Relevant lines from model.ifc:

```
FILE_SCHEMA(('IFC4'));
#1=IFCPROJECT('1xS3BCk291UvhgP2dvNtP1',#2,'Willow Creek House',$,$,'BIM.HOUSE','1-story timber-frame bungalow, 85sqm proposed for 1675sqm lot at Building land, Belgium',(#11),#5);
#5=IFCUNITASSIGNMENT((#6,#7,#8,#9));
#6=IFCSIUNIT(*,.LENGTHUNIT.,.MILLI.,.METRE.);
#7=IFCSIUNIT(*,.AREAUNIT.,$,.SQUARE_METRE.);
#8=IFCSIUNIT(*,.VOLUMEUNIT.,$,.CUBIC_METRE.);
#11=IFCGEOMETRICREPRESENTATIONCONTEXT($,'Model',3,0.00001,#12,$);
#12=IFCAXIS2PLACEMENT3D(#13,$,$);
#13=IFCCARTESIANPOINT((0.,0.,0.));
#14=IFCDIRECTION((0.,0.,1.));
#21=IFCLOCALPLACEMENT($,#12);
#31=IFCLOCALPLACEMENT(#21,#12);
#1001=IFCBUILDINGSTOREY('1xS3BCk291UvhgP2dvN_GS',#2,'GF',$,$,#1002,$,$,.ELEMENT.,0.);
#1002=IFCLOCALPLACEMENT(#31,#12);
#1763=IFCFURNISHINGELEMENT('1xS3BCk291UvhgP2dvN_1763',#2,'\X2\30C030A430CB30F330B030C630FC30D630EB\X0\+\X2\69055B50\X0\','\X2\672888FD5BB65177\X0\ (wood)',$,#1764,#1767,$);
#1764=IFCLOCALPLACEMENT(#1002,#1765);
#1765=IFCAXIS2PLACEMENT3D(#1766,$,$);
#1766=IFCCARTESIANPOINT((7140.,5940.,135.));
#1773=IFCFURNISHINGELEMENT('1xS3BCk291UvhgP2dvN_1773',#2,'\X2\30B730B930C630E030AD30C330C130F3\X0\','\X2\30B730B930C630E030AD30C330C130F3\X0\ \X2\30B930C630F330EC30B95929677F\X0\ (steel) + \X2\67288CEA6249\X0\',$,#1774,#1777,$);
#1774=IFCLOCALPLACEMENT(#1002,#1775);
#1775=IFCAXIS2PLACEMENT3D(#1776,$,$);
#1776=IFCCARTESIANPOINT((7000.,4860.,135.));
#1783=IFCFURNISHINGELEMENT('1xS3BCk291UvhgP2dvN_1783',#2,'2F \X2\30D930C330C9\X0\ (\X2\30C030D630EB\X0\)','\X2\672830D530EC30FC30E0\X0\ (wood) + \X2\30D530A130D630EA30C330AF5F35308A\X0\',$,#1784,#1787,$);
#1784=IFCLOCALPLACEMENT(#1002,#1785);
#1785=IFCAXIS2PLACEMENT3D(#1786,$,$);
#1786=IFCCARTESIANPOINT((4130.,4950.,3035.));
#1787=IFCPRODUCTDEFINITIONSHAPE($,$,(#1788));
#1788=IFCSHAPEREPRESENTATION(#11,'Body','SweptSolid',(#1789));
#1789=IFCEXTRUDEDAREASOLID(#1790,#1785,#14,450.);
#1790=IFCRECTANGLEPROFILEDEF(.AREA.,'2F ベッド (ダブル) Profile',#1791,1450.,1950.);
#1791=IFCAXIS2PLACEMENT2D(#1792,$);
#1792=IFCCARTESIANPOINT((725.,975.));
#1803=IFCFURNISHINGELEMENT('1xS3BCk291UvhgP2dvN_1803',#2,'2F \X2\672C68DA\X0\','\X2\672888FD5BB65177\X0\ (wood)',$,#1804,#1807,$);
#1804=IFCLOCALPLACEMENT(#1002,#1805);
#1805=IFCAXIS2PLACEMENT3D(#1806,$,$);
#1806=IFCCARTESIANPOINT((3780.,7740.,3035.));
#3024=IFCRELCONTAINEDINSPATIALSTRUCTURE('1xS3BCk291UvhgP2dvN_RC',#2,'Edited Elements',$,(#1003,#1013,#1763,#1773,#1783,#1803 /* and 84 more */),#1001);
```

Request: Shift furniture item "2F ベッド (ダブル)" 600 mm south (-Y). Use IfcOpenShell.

```python
import ifcopenshell
import ifcopenshell.api.geometry
import ifcopenshell.util.placement
import ifcopenshell.util.unit

model = ifcopenshell.open("model.ifc")
unit_scale = ifcopenshell.util.unit.calculate_unit_scale(model)

item = model.by_guid("1xS3BCk291UvhgP2dvN_1783")
matrix = ifcopenshell.util.placement.get_local_placement(item.ObjectPlacement)
matrix[1, 3] -= 0.6 / unit_scale
ifcopenshell.api.geometry.edit_object_placement(model, product=item, matrix=matrix, is_si=False)

print(ifcopenshell.util.placement.get_local_placement(item.ObjectPlacement).round(3) + 0.0)

model.write("model_updated.ifc")
```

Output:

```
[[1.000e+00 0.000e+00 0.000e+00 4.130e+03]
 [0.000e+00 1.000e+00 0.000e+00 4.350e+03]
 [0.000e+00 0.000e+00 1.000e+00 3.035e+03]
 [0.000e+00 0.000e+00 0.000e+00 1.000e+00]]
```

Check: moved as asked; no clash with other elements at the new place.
